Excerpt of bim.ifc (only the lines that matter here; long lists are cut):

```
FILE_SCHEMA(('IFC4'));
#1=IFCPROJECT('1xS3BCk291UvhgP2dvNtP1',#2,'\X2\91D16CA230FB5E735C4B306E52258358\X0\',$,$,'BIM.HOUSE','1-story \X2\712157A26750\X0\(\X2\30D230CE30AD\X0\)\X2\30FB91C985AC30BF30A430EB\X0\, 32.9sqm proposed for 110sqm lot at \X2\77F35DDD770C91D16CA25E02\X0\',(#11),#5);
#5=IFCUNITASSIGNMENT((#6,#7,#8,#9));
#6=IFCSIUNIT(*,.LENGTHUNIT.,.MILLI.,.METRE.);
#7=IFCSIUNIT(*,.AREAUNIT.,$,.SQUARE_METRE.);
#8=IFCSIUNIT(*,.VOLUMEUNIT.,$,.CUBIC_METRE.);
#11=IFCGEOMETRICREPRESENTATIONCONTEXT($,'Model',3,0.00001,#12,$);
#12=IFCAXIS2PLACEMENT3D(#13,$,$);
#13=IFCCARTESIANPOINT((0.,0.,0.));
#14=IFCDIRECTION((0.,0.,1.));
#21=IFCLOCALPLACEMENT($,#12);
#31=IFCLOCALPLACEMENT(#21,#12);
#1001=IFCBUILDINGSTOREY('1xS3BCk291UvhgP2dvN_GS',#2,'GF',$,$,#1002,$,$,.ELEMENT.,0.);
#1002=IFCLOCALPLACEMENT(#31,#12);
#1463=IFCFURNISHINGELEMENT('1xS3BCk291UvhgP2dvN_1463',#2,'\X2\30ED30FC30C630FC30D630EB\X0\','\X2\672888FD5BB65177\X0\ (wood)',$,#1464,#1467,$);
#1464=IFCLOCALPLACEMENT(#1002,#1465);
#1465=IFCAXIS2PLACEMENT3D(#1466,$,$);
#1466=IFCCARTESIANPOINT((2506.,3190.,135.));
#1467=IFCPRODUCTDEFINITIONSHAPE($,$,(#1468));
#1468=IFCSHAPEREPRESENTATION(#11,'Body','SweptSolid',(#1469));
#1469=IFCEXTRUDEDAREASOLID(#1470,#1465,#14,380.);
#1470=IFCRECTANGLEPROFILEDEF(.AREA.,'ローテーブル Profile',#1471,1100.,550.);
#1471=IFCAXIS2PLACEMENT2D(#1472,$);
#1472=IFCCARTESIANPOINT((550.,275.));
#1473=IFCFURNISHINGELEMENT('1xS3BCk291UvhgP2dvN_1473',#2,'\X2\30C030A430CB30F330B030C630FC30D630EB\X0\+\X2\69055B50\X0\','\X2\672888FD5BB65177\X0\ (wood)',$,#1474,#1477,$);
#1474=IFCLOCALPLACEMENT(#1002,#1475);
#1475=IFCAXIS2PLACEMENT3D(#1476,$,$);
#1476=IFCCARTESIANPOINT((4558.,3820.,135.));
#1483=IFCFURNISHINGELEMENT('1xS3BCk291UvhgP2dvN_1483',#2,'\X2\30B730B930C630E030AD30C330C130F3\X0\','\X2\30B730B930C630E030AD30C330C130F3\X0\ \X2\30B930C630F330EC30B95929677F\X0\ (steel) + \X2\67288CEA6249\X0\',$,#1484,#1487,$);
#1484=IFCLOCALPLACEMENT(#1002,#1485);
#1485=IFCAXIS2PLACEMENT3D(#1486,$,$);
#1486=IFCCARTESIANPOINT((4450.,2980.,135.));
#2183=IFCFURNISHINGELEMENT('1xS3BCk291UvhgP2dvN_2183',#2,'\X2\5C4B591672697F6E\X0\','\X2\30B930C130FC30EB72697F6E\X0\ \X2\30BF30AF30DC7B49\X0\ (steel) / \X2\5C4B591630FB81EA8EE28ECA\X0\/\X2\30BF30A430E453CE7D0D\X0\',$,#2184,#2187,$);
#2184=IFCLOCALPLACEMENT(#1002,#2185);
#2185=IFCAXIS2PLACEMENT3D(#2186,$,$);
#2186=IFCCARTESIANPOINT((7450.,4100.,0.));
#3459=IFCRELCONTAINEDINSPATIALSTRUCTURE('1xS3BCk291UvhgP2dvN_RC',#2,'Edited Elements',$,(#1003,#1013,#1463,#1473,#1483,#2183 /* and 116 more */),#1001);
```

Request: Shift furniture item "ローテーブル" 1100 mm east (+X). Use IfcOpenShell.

```python
import ifcopenshell
import ifcopenshell.api.geometry
import ifcopenshell.util.placement
import ifcopenshell.util.unit

model = ifcopenshell.open("bim.ifc")
unit_scale = ifcopenshell.util.unit.calculate_unit_scale(model)

item = model.by_id(1463)
matrix = ifcopenshell.util.placement.get_local_placement(item.ObjectPlacement)
matrix[0, 3] += 1.1 / unit_scale
ifcopenshell.api.geometry.edit_object_placement(model, product=item, matrix=matrix, is_si=False)

print(ifcopenshell.util.placement.get_local_placement(item.ObjectPlacement).round(3) + 0.0)

model.write("bim-out.ifc")
```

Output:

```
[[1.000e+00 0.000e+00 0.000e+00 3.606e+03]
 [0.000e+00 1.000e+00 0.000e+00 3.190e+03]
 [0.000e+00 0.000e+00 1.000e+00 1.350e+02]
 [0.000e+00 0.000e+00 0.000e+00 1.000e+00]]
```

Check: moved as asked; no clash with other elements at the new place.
